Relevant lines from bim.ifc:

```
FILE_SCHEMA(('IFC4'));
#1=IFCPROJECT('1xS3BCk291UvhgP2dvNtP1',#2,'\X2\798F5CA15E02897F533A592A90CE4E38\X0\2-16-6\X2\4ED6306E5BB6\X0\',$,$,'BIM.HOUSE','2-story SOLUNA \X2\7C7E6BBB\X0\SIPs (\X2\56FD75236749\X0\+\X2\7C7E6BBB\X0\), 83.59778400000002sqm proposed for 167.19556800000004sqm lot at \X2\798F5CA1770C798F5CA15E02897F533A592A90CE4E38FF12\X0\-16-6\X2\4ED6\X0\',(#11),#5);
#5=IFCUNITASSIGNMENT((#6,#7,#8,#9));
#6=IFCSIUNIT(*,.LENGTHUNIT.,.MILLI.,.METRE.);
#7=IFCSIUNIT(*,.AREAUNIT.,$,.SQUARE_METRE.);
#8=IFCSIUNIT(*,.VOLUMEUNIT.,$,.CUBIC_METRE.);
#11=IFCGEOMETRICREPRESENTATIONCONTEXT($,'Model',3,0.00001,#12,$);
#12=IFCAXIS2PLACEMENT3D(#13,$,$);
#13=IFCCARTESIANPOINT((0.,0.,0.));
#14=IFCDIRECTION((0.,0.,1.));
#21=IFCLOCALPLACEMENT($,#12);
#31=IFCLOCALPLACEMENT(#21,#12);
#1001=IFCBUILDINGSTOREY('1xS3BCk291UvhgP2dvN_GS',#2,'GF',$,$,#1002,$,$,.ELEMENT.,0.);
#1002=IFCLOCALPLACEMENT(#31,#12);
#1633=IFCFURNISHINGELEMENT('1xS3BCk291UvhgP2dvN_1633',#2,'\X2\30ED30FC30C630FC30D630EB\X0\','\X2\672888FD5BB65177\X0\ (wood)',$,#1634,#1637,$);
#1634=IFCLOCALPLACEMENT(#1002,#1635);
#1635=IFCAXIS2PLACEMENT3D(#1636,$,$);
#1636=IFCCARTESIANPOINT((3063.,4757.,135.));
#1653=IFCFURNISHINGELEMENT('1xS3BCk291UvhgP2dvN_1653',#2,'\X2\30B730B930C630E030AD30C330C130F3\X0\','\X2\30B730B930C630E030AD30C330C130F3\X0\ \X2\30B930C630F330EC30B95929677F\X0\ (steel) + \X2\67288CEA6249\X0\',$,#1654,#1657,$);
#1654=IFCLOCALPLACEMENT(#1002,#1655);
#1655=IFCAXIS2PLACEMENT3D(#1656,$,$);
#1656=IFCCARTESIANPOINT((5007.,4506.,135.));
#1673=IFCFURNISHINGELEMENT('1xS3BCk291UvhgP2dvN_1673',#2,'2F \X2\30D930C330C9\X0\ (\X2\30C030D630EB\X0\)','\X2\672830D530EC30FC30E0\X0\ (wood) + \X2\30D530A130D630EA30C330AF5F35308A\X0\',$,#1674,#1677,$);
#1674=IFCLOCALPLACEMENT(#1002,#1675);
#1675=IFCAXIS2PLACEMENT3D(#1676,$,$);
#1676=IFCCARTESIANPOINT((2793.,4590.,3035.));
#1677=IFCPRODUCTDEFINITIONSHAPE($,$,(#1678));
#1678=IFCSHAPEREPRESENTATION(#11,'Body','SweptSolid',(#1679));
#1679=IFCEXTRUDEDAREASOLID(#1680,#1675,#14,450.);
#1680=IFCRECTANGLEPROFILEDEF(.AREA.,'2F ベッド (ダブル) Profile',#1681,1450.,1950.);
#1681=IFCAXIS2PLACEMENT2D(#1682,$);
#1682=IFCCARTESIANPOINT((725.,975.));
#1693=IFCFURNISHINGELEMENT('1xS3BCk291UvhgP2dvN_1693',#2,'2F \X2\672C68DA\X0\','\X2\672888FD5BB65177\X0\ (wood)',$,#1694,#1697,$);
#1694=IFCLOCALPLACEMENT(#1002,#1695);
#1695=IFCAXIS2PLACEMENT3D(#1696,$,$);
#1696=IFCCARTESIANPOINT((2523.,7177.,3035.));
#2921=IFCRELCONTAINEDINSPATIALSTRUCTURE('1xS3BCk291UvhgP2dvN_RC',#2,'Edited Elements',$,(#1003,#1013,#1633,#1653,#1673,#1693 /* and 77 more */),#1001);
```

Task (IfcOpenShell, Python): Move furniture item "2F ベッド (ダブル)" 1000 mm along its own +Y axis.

```python
import ifcopenshell
import ifcopenshell.api.geometry
import ifcopenshell.util.placement
import ifcopenshell.util.unit

model = ifcopenshell.open("bim.ifc")
unit_scale = ifcopenshell.util.unit.calculate_unit_scale(model)

item = model.by_guid("1xS3BCk291UvhgP2dvN_1673")
matrix = ifcopenshell.util.placement.get_local_placement(item.ObjectPlacement)
matrix[:3, 3] += matrix[:3, 1] * 1 / unit_scale
ifcopenshell.api.geometry.edit_object_placement(model, product=item, matrix=matrix, is_si=False)

print(ifcopenshell.util.placement.get_local_placement(item.ObjectPlacement).round(3) + 0.0)

model.write("bim_edited.ifc")
```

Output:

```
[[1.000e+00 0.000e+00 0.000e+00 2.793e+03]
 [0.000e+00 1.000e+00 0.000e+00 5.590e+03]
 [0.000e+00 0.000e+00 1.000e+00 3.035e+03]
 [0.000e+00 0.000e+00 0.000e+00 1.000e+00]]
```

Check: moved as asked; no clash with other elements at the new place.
